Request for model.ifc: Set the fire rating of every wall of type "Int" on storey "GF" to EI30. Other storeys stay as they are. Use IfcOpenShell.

First a look at what the model holds.

```python
import ifcopenshell
import ifcopenshell.util.element

model = ifcopenshell.open("model.ifc")
print(model.schema)
storey = next(s for s in model.by_type("IfcBuildingStorey") if s.Name == "GF")
walls = [e for e in ifcopenshell.util.element.get_decomposition(storey) if e.is_a("IfcWall")]
seen = {}
for e in walls:
    element_type = ifcopenshell.util.element.get_type(e)
    key = (element_type.Name if element_type != e and element_type else None, ifcopenshell.util.element.get_pset(e, "Pset_WallCommon", "FireRating"))
    seen[key] = seen.get(key, 0) + 1
for (name, value), count in sorted(seen.items(), key=str):
    print(count, "x", name, "|", value)
```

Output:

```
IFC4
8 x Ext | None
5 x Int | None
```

```python
import ifcopenshell
import ifcopenshell.api.pset
import ifcopenshell.util.element

model = ifcopenshell.open("model.ifc")

storey = next(s for s in model.by_type("IfcBuildingStorey") if s.Name == "GF")
walls = [e for e in ifcopenshell.util.element.get_decomposition(storey) if e.is_a("IfcWall")]

count = 0
for e in walls:
    element_type = ifcopenshell.util.element.get_type(e)
    if element_type in (None, e) or element_type.Name != "Int":
        continue
    # add_pset returns the element's existing set when there is one.
    pset = ifcopenshell.api.pset.add_pset(model, product=e, name="Pset_WallCommon")
    ifcopenshell.api.pset.edit_pset(model, pset=pset, properties={"FireRating": "EI30"})
    count += 1

print(count, "walls updated")

model.write("model_rev.ifc")
```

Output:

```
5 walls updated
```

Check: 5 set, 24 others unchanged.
